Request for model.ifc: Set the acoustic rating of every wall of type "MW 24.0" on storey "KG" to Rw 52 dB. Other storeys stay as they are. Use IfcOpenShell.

First a look at what the model holds.

```python
import ifcopenshell
import ifcopenshell.util.element

model = ifcopenshell.open("model.ifc")
print(model.schema)
storey = next(s for s in model.by_type("IfcBuildingStorey") if s.Name == "KG")
walls = [e for e in ifcopenshell.util.element.get_decomposition(storey) if e.is_a("IfcWall")]
seen = {}
for e in walls:
    element_type = ifcopenshell.util.element.get_type(e)
    key = (element_type.Name if element_type != e and element_type else None, ifcopenshell.util.element.get_pset(e, "Pset_WallCommon", "AcousticRating"))
    seen[key] = seen.get(key, 0) + 1
for (name, value), count in sorted(seen.items(), key=str):
    print(count, "x", name, "|", value)
```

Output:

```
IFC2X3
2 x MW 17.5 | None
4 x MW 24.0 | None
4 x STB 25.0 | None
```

```python
import ifcopenshell
import ifcopenshell.api.pset
import ifcopenshell.util.element

model = ifcopenshell.open("model.ifc")

storey = next(s for s in model.by_type("IfcBuildingStorey") if s.Name == "KG")
walls = [e for e in ifcopenshell.util.element.get_decomposition(storey) if e.is_a("IfcWall")]

count = 0
for e in walls:
    element_type = ifcopenshell.util.element.get_type(e)
    if element_type in (None, e) or element_type.Name != "MW 24.0":
        continue
    # add_pset returns the element's existing set when there is one.
    pset = ifcopenshell.api.pset.add_pset(model, product=e, name="Pset_WallCommon")
    ifcopenshell.api.pset.edit_pset(model, pset=pset, properties={"AcousticRating": "Rw 52 dB"})
    count += 1

print(count, "walls updated")

model.write("model_v2.ifc")
```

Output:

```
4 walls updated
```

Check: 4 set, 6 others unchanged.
